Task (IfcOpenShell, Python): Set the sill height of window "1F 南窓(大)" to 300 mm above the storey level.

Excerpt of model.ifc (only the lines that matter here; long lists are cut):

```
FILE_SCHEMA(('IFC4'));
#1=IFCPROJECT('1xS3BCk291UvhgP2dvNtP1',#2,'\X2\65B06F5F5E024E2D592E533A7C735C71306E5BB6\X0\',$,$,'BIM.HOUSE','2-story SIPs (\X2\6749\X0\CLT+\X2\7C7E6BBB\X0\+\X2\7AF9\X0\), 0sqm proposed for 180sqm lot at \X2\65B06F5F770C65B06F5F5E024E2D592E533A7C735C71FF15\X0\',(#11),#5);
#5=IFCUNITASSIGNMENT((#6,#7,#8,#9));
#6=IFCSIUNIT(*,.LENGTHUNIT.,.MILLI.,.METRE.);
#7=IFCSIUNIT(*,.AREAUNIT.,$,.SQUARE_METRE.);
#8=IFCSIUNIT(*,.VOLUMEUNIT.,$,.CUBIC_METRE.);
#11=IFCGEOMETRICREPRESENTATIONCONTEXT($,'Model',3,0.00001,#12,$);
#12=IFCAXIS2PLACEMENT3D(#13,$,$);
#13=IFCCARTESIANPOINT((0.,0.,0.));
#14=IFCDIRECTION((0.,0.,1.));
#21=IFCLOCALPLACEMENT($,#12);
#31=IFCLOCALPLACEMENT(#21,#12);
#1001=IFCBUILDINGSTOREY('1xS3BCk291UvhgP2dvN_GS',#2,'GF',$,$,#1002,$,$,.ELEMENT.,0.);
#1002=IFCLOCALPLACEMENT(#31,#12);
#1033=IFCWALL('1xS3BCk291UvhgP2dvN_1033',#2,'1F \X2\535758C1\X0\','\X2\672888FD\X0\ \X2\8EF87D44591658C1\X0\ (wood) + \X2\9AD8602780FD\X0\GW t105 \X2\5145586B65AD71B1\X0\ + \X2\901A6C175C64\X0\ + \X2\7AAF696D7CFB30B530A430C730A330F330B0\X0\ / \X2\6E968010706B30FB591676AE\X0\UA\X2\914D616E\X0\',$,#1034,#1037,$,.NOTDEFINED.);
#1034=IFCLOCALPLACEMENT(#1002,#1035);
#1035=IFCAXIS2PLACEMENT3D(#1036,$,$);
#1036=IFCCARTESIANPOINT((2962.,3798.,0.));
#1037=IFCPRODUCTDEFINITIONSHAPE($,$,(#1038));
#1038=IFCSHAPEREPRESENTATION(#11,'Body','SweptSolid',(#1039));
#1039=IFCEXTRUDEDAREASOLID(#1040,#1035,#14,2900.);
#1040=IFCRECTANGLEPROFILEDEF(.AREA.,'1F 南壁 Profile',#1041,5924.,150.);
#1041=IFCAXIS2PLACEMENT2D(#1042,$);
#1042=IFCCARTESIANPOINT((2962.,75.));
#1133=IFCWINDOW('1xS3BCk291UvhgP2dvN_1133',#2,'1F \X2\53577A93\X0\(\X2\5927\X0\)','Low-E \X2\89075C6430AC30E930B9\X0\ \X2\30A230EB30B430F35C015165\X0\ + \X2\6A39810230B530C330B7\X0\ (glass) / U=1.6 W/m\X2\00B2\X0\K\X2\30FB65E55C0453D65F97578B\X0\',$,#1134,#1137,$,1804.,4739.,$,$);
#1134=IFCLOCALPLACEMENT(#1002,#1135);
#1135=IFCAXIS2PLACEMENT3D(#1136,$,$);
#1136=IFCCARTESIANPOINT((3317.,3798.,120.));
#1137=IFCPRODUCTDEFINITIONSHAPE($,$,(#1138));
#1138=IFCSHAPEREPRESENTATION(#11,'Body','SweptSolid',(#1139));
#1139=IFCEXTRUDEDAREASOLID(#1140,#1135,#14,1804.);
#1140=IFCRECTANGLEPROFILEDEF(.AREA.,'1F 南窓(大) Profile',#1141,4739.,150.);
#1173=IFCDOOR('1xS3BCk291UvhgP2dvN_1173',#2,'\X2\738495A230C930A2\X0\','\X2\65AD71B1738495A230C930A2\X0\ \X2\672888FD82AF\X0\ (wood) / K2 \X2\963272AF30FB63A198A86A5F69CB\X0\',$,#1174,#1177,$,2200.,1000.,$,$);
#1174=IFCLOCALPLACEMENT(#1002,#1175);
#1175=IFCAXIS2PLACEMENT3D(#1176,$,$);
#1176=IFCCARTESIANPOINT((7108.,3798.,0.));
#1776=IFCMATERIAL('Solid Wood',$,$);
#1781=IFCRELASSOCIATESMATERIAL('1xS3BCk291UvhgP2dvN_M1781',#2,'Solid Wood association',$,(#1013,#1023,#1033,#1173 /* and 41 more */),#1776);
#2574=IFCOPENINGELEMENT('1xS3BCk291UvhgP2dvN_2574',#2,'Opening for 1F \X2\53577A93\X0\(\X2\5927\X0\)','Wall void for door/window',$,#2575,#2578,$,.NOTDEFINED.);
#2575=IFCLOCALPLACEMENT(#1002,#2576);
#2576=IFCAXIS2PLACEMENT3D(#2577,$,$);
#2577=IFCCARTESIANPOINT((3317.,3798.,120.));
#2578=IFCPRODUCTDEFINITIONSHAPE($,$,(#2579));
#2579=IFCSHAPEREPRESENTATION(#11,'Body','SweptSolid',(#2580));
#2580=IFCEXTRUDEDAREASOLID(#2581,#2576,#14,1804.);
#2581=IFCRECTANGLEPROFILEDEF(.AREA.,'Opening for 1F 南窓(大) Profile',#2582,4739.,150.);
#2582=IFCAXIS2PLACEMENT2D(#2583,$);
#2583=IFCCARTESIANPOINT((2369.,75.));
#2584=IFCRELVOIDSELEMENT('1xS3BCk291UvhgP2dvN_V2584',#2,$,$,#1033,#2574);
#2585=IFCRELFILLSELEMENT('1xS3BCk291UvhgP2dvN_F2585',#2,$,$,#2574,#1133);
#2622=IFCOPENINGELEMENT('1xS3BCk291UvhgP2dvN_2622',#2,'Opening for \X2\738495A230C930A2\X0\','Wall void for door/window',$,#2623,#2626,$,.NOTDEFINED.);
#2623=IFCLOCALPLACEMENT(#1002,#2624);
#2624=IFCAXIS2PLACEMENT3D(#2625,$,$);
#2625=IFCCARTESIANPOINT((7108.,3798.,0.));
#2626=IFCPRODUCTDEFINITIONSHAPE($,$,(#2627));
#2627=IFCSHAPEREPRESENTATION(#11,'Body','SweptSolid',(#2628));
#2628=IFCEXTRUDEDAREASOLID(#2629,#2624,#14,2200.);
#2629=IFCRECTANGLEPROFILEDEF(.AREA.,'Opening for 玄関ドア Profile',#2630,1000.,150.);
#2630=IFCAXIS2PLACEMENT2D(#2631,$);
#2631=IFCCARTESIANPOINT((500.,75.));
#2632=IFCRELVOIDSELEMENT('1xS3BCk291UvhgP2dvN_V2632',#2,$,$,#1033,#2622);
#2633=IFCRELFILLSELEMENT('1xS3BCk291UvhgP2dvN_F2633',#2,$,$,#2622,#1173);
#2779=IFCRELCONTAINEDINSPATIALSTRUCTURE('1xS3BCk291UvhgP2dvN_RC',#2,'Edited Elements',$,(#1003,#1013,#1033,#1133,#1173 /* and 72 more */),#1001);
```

```python
import numpy as np
import ifcopenshell
import ifcopenshell.api.geometry
import ifcopenshell.geom
import ifcopenshell.util.element
import ifcopenshell.util.placement
import ifcopenshell.util.shape
import ifcopenshell.util.unit

model = ifcopenshell.open("model.ifc")
unit_scale = ifcopenshell.util.unit.calculate_unit_scale(model)

window = model.by_guid("1xS3BCk291UvhgP2dvN_1133")
opening = window.FillsVoids[0].RelatingOpeningElement
storey = ifcopenshell.util.element.get_container(window, ifc_class="IfcBuildingStorey")
level = ifcopenshell.util.placement.get_local_placement(storey.ObjectPlacement)[2, 3]

# The opening's origin need not be at the sill, so measure its lowest point.
shape = ifcopenshell.geom.create_shape(ifcopenshell.geom.settings(), opening)
bottom = ifcopenshell.util.shape.get_shape_bottom_elevation(shape, shape.geometry) / unit_scale
dz = level + 300.0 - bottom

shift = np.array([0.0, 0.0, dz])
# The window is not placed relative to its opening, so move both.
for product in (opening, window):
    matrix = ifcopenshell.util.placement.get_local_placement(product.ObjectPlacement)
    matrix[:3, 3] += shift
    ifcopenshell.api.geometry.edit_object_placement(model, product=product, matrix=matrix, is_si=False)

print(f"moved by {dz * unit_scale:+.3f} m")

model.write("model_updated.ifc")
```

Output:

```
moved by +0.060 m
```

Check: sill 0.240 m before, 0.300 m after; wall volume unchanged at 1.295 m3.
